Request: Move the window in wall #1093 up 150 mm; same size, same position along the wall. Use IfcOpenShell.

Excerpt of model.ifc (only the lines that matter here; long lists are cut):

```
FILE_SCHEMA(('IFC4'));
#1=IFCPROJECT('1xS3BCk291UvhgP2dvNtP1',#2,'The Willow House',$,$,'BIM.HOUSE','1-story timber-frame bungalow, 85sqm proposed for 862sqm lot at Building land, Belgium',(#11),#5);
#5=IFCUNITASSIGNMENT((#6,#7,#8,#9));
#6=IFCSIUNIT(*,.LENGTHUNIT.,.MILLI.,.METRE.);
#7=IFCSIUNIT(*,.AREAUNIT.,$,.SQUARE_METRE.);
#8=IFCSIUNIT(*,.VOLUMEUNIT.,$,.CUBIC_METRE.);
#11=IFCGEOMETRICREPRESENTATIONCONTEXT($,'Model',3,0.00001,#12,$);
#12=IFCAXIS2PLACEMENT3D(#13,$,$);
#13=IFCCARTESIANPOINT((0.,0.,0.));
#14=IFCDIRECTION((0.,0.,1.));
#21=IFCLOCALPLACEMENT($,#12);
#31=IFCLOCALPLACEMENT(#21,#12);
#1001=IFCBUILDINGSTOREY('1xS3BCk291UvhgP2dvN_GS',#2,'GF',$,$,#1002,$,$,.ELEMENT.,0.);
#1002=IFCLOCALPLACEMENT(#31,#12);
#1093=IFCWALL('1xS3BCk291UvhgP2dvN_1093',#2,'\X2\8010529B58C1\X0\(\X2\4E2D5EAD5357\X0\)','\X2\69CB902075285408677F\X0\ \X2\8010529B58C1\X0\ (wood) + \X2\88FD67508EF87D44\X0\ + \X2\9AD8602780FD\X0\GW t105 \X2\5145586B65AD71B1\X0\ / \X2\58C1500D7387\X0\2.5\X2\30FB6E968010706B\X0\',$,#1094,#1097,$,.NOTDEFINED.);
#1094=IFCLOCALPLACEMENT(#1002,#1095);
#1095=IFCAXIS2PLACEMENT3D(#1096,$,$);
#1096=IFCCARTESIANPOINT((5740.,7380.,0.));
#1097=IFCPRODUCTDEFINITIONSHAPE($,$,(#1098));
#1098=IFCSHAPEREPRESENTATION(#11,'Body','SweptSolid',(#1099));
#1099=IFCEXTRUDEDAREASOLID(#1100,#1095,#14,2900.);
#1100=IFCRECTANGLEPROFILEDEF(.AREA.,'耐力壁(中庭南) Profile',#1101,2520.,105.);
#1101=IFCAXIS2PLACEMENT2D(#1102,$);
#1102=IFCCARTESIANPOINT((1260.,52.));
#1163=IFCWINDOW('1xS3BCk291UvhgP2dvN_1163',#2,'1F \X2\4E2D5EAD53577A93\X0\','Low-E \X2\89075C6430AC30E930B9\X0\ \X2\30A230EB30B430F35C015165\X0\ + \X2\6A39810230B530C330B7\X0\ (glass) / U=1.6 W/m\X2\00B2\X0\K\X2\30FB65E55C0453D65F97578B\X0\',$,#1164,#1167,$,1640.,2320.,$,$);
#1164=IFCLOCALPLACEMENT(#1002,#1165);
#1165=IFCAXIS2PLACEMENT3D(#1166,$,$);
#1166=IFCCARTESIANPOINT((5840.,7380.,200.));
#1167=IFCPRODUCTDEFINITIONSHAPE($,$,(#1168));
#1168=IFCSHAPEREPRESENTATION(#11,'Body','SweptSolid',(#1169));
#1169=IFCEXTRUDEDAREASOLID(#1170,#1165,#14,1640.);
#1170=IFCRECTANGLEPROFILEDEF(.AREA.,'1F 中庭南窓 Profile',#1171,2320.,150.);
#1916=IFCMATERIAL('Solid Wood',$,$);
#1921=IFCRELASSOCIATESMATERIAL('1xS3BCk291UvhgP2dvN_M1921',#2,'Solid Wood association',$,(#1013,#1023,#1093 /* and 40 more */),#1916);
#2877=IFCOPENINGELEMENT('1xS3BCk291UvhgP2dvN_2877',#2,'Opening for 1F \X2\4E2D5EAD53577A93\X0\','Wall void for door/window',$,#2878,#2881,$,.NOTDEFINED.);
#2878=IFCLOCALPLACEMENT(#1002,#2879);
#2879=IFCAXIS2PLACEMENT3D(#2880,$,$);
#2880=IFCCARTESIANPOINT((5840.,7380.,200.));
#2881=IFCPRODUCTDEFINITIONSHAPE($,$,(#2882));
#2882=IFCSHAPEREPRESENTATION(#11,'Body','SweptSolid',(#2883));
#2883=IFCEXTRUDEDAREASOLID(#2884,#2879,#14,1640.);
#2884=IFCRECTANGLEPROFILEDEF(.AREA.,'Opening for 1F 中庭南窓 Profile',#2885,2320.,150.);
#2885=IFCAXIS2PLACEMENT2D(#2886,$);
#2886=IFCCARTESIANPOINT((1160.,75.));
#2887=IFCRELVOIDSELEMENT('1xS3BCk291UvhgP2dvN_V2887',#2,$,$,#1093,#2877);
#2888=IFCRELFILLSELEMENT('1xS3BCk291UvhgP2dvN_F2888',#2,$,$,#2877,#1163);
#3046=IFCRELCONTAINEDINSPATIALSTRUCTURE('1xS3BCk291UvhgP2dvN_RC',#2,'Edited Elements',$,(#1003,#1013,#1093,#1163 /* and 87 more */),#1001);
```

```python
import numpy as np
import ifcopenshell
import ifcopenshell.api.geometry
import ifcopenshell.util.placement
import ifcopenshell.util.unit

model = ifcopenshell.open("model.ifc")
unit_scale = ifcopenshell.util.unit.calculate_unit_scale(model)

window = model.by_guid("1xS3BCk291UvhgP2dvN_1163")
opening = window.FillsVoids[0].RelatingOpeningElement
dz = 0.15 / unit_scale

shift = np.array([0.0, 0.0, dz])
# The window is not placed relative to its opening, so move both.
for product in (opening, window):
    matrix = ifcopenshell.util.placement.get_local_placement(product.ObjectPlacement)
    matrix[:3, 3] += shift
    ifcopenshell.api.geometry.edit_object_placement(model, product=product, matrix=matrix, is_si=False)

print(f"moved by {dz * unit_scale:+.3f} m")

model.write("model-out.ifc")
```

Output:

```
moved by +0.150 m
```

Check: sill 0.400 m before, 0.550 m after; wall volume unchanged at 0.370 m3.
